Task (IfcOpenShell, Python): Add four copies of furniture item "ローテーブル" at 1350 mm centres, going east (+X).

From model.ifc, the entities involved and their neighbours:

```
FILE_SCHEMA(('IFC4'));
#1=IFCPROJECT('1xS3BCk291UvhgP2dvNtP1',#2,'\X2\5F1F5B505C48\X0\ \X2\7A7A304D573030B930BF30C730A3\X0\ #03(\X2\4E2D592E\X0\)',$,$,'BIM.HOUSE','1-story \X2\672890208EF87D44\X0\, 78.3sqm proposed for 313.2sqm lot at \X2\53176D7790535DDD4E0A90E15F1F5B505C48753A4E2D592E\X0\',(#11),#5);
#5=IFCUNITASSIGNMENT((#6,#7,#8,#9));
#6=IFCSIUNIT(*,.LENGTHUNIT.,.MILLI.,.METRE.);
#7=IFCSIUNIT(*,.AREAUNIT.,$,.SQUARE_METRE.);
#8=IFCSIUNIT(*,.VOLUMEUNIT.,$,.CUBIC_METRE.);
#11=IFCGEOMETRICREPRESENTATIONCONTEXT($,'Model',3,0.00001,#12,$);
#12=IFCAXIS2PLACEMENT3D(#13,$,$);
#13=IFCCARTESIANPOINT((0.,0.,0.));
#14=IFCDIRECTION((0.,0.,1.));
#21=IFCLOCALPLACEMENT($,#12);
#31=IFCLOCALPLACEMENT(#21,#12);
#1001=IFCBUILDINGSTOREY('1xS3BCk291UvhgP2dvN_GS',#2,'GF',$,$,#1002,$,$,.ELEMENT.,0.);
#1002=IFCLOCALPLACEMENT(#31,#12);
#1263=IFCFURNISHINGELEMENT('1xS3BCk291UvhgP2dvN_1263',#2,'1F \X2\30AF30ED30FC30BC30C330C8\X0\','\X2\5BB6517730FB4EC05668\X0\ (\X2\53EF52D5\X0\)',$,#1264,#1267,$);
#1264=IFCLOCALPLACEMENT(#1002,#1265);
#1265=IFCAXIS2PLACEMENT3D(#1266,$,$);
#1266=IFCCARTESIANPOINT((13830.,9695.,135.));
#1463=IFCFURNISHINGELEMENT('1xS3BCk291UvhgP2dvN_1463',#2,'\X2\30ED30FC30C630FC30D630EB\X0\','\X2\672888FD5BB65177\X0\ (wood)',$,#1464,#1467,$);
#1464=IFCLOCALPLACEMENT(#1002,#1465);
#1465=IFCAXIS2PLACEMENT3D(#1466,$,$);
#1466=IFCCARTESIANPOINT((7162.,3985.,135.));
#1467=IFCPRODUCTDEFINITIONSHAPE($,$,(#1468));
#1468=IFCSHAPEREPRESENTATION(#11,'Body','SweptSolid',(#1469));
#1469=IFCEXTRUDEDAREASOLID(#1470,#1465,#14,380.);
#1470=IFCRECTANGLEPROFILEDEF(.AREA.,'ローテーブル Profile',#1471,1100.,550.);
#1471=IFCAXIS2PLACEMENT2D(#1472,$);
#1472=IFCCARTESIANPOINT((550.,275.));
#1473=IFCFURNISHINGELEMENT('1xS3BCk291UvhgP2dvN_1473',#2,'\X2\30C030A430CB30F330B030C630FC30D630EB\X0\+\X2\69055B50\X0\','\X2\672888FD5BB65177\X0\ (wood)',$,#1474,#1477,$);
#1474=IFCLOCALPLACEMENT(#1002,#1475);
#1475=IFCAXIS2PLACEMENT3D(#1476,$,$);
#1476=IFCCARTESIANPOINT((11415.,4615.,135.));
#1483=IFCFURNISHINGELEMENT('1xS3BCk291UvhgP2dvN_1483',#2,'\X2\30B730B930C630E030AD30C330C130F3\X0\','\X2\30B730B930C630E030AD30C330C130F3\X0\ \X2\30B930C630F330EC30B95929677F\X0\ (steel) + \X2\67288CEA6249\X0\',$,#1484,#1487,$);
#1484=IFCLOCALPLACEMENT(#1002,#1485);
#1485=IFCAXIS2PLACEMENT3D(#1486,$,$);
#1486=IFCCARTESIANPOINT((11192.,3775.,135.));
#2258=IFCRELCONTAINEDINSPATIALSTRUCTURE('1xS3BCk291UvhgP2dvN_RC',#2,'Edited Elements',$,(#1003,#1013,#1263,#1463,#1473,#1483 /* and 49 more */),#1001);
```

```python
import numpy as np
import ifcopenshell
import ifcopenshell.api.geometry
import ifcopenshell.api.root
import ifcopenshell.util.element
import ifcopenshell.util.placement

model = ifcopenshell.open("model.ifc")


def reuse_history(source, copy):
    """copy_class also copies each property set's owner history, people and application; keep the originals."""
    for rel in copy.IsDefinedBy:
        if rel.is_a("IfcRelDefinesByProperties") and (history := rel.RelatingPropertyDefinition.OwnerHistory):
            rel.RelatingPropertyDefinition.OwnerHistory = source.OwnerHistory
            ifcopenshell.util.element.remove_deep2(model, history)


source = model.by_id(1463)
base = ifcopenshell.util.placement.get_local_placement(source.ObjectPlacement)
step = np.array([1.0, 0.0, 0.0]) * 1350.0

for i in range(1, 5):
    copy = ifcopenshell.api.root.copy_class(model, product=source)
    copy.Representation = ifcopenshell.util.element.copy_deep(
        model, source.Representation, exclude=["IfcGeometricRepresentationContext", "IfcRepresentationMap"]
    )
    reuse_history(source, copy)
    matrix = base.copy()
    matrix[:3, 3] += i * step
    print("added at", matrix[:3, 3].round(3) + 0.0)
    ifcopenshell.api.geometry.edit_object_placement(model, product=copy, matrix=matrix, is_si=False)

model.write("model_edited.ifc")
```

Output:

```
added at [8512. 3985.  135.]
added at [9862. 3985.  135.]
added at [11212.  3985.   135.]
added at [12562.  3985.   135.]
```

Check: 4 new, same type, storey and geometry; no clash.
